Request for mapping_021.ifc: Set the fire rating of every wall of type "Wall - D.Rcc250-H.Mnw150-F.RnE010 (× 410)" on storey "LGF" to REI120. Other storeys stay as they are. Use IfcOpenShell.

First a look at what the model holds.

```python
import ifcopenshell
import ifcopenshell.util.element

model = ifcopenshell.open("mapping_021.ifc")
print(model.schema)
storey = next(s for s in model.by_type("IfcBuildingStorey") if s.Name == "LGF")
walls = [e for e in ifcopenshell.util.element.get_decomposition(storey) if e.is_a("IfcWall")]
seen = {}
for e in walls:
    element_type = ifcopenshell.util.element.get_type(e)
    key = (element_type.Name if element_type != e and element_type else None, ifcopenshell.util.element.get_pset(e, "Pset_WallCommon", "FireRating"))
    seen[key] = seen.get(key, 0) + 1
for (name, value), count in sorted(seen.items(), key=str):
    print(count, "x", name, "|", value)
```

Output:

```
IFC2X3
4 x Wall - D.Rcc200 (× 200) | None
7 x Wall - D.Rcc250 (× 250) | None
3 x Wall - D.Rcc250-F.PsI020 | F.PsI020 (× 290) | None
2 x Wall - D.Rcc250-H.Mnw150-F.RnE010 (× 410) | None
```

```python
import ifcopenshell
import ifcopenshell.api.pset
import ifcopenshell.util.element

model = ifcopenshell.open("mapping_021.ifc")

storey = next(s for s in model.by_type("IfcBuildingStorey") if s.Name == "LGF")
walls = [e for e in ifcopenshell.util.element.get_decomposition(storey) if e.is_a("IfcWall")]

count = 0
for e in walls:
    element_type = ifcopenshell.util.element.get_type(e)
    if element_type in (None, e) or element_type.Name != "Wall - D.Rcc250-H.Mnw150-F.RnE010 (× 410)":
        continue
    # add_pset returns the element's existing set when there is one.
    pset = ifcopenshell.api.pset.add_pset(model, product=e, name="Pset_WallCommon")
    ifcopenshell.api.pset.edit_pset(model, pset=pset, properties={"FireRating": "REI120"})
    count += 1

print(count, "walls updated")

model.write("mapping_021_rev.ifc")
```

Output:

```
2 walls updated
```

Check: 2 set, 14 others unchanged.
